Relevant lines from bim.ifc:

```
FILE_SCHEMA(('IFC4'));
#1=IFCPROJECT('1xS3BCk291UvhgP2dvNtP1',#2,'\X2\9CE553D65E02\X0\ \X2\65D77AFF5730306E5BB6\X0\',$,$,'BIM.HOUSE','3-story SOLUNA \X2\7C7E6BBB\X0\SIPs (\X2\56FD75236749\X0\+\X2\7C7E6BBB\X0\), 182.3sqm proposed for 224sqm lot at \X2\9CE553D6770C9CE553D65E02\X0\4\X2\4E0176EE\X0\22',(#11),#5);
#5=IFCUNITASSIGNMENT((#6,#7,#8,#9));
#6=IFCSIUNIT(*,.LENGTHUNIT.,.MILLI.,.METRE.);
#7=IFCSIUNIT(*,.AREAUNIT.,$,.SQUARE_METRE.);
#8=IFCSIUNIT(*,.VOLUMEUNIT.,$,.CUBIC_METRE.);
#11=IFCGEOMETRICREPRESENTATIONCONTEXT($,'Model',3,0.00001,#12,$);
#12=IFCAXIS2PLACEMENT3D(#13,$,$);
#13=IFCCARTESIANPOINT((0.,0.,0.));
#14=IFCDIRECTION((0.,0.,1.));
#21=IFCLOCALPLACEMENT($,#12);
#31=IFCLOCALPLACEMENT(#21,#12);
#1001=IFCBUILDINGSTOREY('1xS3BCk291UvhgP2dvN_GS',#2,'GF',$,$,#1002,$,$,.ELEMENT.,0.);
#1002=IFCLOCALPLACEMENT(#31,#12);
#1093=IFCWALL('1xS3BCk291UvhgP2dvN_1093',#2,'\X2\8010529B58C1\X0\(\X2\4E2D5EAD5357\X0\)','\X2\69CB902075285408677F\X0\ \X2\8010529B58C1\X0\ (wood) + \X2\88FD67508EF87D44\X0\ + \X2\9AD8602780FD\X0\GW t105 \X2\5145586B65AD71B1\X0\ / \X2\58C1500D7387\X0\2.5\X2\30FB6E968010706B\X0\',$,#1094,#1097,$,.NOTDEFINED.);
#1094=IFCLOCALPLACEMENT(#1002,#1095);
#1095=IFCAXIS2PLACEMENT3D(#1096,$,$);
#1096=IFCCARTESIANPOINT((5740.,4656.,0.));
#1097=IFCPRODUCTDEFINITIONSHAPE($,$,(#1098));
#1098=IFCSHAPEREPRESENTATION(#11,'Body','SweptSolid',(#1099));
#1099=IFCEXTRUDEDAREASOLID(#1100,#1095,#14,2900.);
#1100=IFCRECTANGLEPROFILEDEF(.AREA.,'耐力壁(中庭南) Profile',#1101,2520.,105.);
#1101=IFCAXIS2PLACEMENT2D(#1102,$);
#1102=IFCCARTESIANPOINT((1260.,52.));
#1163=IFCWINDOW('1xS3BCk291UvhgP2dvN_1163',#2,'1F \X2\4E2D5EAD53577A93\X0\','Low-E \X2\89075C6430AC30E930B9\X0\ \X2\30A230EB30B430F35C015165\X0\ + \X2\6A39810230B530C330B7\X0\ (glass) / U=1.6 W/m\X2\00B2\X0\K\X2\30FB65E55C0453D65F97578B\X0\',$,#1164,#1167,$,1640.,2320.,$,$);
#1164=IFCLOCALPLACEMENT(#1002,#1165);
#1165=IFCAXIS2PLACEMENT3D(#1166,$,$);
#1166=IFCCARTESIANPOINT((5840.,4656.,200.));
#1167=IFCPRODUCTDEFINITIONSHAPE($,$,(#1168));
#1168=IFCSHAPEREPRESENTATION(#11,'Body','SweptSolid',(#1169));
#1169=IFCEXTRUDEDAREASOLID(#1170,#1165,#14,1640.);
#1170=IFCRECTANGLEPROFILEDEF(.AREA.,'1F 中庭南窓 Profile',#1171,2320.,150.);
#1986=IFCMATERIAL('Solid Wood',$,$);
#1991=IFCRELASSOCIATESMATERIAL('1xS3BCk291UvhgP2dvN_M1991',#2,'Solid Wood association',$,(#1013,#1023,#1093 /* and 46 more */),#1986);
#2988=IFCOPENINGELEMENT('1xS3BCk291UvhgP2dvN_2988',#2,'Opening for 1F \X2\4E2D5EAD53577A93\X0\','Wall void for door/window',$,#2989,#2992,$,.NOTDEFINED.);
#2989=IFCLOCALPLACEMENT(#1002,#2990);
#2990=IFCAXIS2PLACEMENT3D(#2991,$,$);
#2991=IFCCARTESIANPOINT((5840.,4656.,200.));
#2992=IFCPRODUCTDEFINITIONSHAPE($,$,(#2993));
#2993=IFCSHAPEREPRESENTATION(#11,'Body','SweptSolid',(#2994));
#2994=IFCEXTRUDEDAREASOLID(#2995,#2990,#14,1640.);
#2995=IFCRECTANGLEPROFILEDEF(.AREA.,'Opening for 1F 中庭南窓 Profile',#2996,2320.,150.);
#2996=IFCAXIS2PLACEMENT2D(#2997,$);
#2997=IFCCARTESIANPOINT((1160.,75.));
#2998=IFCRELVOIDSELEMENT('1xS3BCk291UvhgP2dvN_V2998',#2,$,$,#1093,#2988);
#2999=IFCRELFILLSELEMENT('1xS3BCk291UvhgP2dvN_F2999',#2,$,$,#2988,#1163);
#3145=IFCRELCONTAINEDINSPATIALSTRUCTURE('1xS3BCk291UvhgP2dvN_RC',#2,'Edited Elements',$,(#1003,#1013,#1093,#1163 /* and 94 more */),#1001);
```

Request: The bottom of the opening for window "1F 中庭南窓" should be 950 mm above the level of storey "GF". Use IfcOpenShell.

```python
import numpy as np
import ifcopenshell
import ifcopenshell.api.geometry
import ifcopenshell.geom
import ifcopenshell.util.element
import ifcopenshell.util.placement
import ifcopenshell.util.shape
import ifcopenshell.util.unit

model = ifcopenshell.open("bim.ifc")
unit_scale = ifcopenshell.util.unit.calculate_unit_scale(model)

window = model.by_guid("1xS3BCk291UvhgP2dvN_1163")
opening = window.FillsVoids[0].RelatingOpeningElement
storey = ifcopenshell.util.element.get_container(window, ifc_class="IfcBuildingStorey")
level = ifcopenshell.util.placement.get_local_placement(storey.ObjectPlacement)[2, 3]

# The opening's origin need not be at the sill, so measure its lowest point.
shape = ifcopenshell.geom.create_shape(ifcopenshell.geom.settings(), opening)
bottom = ifcopenshell.util.shape.get_shape_bottom_elevation(shape, shape.geometry) / unit_scale
dz = level + 0.95 / unit_scale - bottom

shift = np.array([0.0, 0.0, dz])
# The window is not placed relative to its opening, so move both.
for product in (opening, window):
    matrix = ifcopenshell.util.placement.get_local_placement(product.ObjectPlacement)
    matrix[:3, 3] += shift
    ifcopenshell.api.geometry.edit_object_placement(model, product=product, matrix=matrix, is_si=False)

print(f"moved by {dz * unit_scale:+.3f} m")

model.write("bim_rev.ifc")
```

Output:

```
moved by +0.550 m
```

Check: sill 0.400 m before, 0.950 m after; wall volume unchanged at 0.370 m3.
